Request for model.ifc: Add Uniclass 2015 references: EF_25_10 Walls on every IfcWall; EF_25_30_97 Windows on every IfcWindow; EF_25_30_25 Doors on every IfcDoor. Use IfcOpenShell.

First a look at what the model holds.

```python
import ifcopenshell

model = ifcopenshell.open("model.ifc")
print(model.schema)
print("classifications:", [c.Name for c in model.by_type("IfcClassification")])
for ifc_class in ("IfcDoor", "IfcRoof", "IfcStair", "IfcWall", "IfcWindow"):
    print(ifc_class, len(model.by_type(ifc_class)))
```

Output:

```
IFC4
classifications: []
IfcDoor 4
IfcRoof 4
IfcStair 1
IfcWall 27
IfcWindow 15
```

```python
import ifcopenshell
import ifcopenshell.api.classification

model = ifcopenshell.open("model.ifc")

system = ifcopenshell.api.classification.add_classification(model, classification="Uniclass 2015")

codes = {
    "IfcWall": ("EF_25_10", "Walls"),
    "IfcWindow": ("EF_25_30_97", "Windows"),
    "IfcDoor": ("EF_25_30_25", "Doors"),
}
for ifc_class, (code, name) in codes.items():
    products = model.by_type(ifc_class)
    ifcopenshell.api.classification.add_reference(
        model, products=products, classification=system, identification=code, name=name
    )
    print(code, len(products))

model.write("model-out.ifc")
```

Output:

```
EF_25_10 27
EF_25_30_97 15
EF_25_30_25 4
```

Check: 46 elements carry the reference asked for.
